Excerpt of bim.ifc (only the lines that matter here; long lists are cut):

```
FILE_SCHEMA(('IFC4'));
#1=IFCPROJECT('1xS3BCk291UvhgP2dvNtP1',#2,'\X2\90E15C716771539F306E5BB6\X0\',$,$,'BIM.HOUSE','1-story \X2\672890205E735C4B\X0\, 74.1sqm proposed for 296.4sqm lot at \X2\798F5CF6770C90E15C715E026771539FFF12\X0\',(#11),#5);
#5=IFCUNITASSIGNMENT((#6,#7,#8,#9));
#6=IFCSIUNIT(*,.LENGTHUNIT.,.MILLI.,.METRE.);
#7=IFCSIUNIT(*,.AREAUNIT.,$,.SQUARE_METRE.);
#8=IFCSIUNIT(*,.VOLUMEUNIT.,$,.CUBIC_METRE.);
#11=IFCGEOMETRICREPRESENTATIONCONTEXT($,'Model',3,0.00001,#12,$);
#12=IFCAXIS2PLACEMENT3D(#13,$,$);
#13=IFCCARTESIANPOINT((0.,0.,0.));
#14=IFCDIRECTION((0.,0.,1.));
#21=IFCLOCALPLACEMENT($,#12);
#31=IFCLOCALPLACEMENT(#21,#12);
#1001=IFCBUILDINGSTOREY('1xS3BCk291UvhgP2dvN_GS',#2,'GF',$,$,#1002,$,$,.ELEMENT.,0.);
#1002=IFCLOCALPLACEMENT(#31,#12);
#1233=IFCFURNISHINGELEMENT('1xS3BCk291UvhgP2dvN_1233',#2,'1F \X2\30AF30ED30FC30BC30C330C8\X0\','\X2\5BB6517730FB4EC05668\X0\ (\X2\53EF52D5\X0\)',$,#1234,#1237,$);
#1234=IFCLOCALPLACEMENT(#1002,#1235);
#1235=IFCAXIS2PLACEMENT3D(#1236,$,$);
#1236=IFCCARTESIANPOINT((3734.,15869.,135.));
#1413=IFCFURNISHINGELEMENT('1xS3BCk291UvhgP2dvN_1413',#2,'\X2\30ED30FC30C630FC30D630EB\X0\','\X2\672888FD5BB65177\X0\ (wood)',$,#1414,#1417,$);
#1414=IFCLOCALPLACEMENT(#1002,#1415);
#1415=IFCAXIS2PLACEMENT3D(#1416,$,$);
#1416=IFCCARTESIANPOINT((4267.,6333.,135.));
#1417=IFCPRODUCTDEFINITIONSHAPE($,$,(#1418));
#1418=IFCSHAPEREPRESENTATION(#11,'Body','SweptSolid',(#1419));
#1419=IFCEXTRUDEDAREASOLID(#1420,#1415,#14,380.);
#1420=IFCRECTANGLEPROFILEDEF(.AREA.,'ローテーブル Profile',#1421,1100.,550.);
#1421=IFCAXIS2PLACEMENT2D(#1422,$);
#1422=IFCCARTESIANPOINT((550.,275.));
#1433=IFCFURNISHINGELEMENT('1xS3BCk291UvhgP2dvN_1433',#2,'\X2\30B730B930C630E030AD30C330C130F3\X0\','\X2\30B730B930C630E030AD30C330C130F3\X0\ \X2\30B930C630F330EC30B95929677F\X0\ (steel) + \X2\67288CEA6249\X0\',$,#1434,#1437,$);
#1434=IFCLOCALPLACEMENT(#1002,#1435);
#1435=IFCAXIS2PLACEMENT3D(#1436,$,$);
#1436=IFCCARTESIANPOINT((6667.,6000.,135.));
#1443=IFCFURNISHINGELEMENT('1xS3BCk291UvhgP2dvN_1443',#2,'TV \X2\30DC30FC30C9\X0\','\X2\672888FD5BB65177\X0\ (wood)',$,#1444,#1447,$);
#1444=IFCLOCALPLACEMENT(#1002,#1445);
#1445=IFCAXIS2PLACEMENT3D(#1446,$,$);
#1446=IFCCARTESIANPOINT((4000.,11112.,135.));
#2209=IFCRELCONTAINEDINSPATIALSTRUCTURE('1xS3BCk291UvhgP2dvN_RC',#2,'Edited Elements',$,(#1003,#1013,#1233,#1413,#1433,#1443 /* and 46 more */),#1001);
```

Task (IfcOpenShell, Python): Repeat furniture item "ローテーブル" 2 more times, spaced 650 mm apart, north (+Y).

```python
import numpy as np
import ifcopenshell
import ifcopenshell.api.geometry
import ifcopenshell.api.root
import ifcopenshell.util.element
import ifcopenshell.util.placement

model = ifcopenshell.open("bim.ifc")


def reuse_history(source, copy):
    """copy_class also copies each property set's owner history, people and application; keep the originals."""
    for rel in copy.IsDefinedBy:
        if rel.is_a("IfcRelDefinesByProperties") and (history := rel.RelatingPropertyDefinition.OwnerHistory):
            rel.RelatingPropertyDefinition.OwnerHistory = source.OwnerHistory
            ifcopenshell.util.element.remove_deep2(model, history)


source = model.by_id(1413)
base = ifcopenshell.util.placement.get_local_placement(source.ObjectPlacement)
step = np.array([0.0, 1.0, 0.0]) * 650.0

for i in range(1, 3):
    copy = ifcopenshell.api.root.copy_class(model, product=source)
    copy.Representation = ifcopenshell.util.element.copy_deep(
        model, source.Representation, exclude=["IfcGeometricRepresentationContext", "IfcRepresentationMap"]
    )
    reuse_history(source, copy)
    matrix = base.copy()
    matrix[:3, 3] += i * step
    print("added at", matrix[:3, 3].round(3) + 0.0)
    ifcopenshell.api.geometry.edit_object_placement(model, product=copy, matrix=matrix, is_si=False)

model.write("bim_edited.ifc")
```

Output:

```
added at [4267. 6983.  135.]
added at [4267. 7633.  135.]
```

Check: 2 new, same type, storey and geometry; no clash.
